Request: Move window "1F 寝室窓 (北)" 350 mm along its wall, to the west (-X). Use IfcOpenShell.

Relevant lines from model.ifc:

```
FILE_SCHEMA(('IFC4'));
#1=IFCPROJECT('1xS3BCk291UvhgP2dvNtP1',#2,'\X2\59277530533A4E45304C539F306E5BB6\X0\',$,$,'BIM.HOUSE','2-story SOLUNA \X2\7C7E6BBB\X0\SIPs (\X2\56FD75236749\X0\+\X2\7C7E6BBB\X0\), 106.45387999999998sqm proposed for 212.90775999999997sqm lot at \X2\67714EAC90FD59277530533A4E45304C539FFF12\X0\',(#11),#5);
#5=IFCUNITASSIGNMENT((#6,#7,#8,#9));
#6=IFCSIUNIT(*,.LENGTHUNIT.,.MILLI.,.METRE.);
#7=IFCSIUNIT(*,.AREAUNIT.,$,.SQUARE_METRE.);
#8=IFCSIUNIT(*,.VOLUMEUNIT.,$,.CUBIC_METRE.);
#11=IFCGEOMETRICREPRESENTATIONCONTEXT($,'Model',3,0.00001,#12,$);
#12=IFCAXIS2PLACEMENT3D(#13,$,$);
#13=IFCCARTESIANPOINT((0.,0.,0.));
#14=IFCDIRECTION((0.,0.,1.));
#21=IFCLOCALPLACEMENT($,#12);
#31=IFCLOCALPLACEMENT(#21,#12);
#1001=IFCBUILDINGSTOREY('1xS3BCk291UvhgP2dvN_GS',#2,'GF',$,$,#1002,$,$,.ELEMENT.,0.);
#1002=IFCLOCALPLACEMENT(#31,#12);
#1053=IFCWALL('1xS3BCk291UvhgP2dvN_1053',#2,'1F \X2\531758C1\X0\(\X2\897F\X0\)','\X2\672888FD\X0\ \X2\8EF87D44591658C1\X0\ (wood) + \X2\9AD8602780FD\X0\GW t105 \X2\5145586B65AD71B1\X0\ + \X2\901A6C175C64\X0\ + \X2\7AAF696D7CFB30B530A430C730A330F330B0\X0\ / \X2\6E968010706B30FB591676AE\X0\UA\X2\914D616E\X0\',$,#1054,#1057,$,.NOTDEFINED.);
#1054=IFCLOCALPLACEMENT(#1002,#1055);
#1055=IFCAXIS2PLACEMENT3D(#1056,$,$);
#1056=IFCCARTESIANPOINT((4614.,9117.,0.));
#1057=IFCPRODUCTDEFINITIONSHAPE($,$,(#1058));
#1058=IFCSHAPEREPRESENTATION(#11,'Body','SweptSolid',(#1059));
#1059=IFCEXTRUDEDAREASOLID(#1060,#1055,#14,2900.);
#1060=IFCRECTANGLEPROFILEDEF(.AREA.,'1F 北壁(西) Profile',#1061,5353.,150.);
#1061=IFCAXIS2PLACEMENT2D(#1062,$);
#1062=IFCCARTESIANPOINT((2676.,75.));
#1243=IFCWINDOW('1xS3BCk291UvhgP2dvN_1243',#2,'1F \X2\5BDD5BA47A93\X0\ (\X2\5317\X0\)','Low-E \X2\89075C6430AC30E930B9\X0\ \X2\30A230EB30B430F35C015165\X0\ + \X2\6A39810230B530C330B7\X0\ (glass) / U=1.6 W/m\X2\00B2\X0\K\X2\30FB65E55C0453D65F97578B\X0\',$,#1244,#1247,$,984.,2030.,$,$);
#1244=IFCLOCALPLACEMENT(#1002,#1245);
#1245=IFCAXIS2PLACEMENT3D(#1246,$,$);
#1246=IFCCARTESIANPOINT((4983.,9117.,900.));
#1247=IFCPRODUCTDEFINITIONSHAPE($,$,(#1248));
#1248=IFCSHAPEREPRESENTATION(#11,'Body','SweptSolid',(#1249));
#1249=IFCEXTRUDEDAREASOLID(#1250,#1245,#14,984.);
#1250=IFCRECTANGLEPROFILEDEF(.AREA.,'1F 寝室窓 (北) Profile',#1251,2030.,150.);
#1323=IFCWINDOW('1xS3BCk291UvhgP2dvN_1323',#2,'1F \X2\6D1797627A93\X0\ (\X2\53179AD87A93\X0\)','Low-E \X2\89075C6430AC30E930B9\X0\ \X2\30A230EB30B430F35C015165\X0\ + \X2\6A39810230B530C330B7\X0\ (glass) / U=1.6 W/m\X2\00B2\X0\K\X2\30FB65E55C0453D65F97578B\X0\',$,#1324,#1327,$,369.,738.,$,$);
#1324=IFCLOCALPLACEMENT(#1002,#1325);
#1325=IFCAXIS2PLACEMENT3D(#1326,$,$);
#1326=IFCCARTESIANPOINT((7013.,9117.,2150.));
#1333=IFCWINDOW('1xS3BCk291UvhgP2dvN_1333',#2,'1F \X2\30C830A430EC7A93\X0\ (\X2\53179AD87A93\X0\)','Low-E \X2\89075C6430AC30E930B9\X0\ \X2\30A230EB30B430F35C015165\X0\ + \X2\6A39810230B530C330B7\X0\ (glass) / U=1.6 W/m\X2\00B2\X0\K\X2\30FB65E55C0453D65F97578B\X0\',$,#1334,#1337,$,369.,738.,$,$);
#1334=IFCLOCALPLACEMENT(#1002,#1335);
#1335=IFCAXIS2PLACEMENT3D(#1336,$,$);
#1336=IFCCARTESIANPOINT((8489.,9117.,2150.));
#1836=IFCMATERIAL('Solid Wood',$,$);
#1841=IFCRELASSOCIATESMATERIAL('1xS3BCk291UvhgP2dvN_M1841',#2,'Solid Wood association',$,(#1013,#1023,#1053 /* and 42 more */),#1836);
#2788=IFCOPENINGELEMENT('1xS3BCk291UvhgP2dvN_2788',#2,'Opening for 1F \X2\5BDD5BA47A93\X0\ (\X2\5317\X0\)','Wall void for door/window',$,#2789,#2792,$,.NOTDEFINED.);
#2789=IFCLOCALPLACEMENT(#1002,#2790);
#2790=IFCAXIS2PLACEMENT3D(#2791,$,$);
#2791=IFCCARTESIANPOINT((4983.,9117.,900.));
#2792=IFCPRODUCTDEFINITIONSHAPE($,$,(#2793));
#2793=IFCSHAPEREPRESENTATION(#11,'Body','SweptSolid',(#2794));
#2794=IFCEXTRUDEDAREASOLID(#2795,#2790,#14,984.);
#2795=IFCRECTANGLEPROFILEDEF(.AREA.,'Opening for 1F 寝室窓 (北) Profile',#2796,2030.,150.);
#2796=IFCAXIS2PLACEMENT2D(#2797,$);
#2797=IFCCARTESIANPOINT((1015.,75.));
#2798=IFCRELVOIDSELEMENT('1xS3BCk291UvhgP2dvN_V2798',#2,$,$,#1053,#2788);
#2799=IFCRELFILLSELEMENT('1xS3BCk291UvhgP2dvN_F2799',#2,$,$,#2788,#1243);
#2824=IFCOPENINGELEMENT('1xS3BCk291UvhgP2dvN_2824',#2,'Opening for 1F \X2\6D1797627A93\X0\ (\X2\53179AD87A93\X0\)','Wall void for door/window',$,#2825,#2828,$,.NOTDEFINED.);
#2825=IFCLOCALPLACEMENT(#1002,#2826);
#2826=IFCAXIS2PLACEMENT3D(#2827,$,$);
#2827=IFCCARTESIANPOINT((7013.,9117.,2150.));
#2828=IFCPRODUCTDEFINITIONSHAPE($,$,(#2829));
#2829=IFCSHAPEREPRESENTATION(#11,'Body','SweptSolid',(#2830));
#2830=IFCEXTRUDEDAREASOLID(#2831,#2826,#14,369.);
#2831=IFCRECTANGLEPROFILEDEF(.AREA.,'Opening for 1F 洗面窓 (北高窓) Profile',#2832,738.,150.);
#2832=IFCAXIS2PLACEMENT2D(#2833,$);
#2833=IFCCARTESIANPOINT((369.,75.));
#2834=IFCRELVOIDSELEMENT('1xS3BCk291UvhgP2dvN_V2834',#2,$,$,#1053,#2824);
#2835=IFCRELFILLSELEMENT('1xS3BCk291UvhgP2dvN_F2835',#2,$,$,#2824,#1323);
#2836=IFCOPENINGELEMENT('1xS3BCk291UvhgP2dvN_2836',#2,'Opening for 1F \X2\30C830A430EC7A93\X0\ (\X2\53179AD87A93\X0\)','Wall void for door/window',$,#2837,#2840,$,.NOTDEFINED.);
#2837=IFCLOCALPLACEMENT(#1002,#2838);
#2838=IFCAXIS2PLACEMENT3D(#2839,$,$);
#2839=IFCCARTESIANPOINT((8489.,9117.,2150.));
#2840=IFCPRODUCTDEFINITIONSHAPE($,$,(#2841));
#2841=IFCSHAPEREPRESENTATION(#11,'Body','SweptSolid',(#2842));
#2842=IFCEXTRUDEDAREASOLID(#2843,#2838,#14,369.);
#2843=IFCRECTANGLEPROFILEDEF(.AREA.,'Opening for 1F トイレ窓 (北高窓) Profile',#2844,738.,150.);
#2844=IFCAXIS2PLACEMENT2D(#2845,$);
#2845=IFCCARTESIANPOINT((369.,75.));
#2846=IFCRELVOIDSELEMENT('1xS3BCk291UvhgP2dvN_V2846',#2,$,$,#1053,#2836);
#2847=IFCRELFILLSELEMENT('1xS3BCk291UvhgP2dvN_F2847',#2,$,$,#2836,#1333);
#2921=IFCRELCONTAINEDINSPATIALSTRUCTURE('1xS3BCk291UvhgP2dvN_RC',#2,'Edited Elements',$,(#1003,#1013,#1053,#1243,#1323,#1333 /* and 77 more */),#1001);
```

```python
import ifcopenshell
import ifcopenshell.api.geometry
import ifcopenshell.util.placement
import ifcopenshell.util.unit

model = ifcopenshell.open("model.ifc")
unit_scale = ifcopenshell.util.unit.calculate_unit_scale(model)

window = model.by_guid("1xS3BCk291UvhgP2dvN_1243")
opening = window.FillsVoids[0].RelatingOpeningElement
wall = opening.VoidsElements[0].RelatingBuildingElement

wall_matrix = ifcopenshell.util.placement.get_local_placement(wall.ObjectPlacement)
shift = wall_matrix[:3, 0] * -0.35 / unit_scale
before = ifcopenshell.util.placement.get_local_placement(window.ObjectPlacement)[:3, 3].copy()

# The window is not placed relative to its opening, so move both.
for product in (opening, window):
    matrix = ifcopenshell.util.placement.get_local_placement(product.ObjectPlacement)
    matrix[:3, 3] += shift
    ifcopenshell.api.geometry.edit_object_placement(model, product=product, matrix=matrix, is_si=False)

after = ifcopenshell.util.placement.get_local_placement(window.ObjectPlacement)[:3, 3]
print("window moved by", (after - before).round(3) + 0.0)

model.write("model-out.ifc")
```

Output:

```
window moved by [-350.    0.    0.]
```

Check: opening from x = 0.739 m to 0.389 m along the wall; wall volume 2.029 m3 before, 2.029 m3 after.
